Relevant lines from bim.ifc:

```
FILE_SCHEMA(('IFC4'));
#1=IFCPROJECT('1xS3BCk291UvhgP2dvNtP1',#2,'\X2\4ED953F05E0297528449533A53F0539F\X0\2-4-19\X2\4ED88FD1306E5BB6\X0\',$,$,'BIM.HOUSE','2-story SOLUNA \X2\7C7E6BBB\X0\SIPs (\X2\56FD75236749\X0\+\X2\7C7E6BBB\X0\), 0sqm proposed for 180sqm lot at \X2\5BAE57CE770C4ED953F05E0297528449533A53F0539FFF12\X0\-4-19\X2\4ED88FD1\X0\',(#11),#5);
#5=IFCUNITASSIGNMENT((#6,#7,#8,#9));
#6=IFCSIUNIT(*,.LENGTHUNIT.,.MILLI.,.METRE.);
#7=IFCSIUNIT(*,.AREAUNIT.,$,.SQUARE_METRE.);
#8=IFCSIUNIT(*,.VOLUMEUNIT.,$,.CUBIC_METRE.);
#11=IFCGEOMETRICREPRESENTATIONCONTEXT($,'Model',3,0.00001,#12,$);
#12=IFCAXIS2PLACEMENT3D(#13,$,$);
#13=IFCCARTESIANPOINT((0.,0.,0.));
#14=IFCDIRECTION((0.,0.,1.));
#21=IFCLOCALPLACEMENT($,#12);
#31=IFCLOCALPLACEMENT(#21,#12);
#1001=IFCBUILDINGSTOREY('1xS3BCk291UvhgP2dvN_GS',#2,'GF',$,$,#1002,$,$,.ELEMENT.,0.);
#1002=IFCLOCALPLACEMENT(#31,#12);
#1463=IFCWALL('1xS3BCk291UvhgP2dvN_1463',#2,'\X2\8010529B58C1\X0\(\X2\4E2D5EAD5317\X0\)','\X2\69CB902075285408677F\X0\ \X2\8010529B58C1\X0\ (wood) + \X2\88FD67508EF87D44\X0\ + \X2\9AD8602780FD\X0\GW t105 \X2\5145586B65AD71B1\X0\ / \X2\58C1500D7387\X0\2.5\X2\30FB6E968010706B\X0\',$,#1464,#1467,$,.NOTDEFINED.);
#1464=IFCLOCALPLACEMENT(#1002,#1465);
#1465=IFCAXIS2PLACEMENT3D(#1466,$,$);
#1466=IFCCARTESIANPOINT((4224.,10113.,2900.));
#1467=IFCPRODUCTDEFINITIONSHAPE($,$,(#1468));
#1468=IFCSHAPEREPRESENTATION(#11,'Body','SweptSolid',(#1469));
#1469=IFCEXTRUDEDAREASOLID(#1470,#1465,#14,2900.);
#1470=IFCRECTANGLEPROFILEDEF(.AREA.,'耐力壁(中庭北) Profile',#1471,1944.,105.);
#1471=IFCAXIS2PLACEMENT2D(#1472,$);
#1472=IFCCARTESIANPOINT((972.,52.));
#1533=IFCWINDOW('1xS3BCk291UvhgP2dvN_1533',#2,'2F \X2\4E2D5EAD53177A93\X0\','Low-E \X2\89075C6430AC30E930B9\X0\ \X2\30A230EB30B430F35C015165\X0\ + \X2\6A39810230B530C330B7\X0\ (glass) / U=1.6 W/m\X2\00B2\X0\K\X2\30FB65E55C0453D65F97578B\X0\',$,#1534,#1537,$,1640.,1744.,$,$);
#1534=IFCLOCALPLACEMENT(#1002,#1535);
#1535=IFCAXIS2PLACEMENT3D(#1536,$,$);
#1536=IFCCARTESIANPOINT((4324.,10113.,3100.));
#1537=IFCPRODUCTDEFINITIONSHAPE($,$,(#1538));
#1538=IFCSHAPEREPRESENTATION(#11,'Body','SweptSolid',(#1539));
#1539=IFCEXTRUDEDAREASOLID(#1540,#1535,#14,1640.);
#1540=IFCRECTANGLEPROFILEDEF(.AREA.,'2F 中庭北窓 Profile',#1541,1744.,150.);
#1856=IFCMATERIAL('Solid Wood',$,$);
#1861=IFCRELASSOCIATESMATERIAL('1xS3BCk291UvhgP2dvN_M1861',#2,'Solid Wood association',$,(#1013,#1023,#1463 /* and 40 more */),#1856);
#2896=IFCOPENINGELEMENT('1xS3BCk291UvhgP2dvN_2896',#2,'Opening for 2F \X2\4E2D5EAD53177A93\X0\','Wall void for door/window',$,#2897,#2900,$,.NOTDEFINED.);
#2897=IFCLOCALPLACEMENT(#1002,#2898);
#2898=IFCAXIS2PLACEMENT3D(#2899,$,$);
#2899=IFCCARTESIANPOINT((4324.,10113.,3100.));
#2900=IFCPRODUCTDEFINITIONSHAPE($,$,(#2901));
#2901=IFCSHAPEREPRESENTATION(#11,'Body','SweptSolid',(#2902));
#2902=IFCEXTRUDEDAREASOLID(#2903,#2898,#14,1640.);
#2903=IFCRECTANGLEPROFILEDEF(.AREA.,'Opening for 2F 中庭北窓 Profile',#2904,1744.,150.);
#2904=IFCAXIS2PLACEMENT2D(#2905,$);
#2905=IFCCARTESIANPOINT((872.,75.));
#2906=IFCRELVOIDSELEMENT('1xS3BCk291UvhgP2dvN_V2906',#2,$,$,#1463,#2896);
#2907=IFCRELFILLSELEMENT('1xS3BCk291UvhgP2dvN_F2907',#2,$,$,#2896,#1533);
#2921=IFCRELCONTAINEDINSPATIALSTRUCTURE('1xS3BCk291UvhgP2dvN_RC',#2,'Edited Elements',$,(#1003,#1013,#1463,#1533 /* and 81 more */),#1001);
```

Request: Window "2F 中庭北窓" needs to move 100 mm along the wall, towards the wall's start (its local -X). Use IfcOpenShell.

```python
import ifcopenshell
import ifcopenshell.api.geometry
import ifcopenshell.util.placement

model = ifcopenshell.open("bim.ifc")

window = model.by_guid("1xS3BCk291UvhgP2dvN_1533")
opening = window.FillsVoids[0].RelatingOpeningElement
wall = opening.VoidsElements[0].RelatingBuildingElement

wall_matrix = ifcopenshell.util.placement.get_local_placement(wall.ObjectPlacement)
shift = wall_matrix[:3, 0] * -100.0
before = ifcopenshell.util.placement.get_local_placement(window.ObjectPlacement)[:3, 3].copy()

# The window is not placed relative to its opening, so move both.
for product in (opening, window):
    matrix = ifcopenshell.util.placement.get_local_placement(product.ObjectPlacement)
    matrix[:3, 3] += shift
    ifcopenshell.api.geometry.edit_object_placement(model, product=product, matrix=matrix, is_si=False)

after = ifcopenshell.util.placement.get_local_placement(window.ObjectPlacement)[:3, 3]
print("window moved by", (after - before).round(3) + 0.0)

model.write("bim-out.ifc")
```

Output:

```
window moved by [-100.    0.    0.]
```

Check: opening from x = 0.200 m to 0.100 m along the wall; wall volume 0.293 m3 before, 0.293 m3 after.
